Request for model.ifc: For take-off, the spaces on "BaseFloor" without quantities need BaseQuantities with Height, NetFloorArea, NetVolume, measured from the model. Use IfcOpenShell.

First a look at what the model holds.

```python
import ifcopenshell
import ifcopenshell.util.element
import ifcopenshell.util.unit

model = ifcopenshell.open("model.ifc")
print(model.schema)
for unit_type in ("LENGTHUNIT", "AREAUNIT", "VOLUMEUNIT"):
    print(unit_type, ifcopenshell.util.unit.calculate_unit_scale(model, unit_type))
storey = next(s for s in model.by_type("IfcBuildingStorey") if s.Name == "BaseFloor")
spaces = [e for e in ifcopenshell.util.element.get_decomposition(storey) if e.is_a("IfcSpace")]
for e in sorted(spaces, key=lambda e: e.id()):
    print(e.id(), e.is_a(), e.Name, list(ifcopenshell.util.element.get_psets(e, qtos_only=True)), sep=" | ")
```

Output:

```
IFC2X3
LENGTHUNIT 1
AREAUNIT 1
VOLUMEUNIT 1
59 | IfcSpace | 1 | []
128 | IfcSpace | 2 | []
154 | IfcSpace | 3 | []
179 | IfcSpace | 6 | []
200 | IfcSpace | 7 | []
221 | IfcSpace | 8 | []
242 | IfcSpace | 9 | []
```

```python
import ifcopenshell
import ifcopenshell.api.pset
import ifcopenshell.geom
import ifcopenshell.util.element
import ifcopenshell.util.shape
import ifcopenshell.util.unit

model = ifcopenshell.open("model.ifc")
unit_scale = ifcopenshell.util.unit.calculate_unit_scale(model)
area_scale = ifcopenshell.util.unit.calculate_unit_scale(model, "AREAUNIT")
volume_scale = ifcopenshell.util.unit.calculate_unit_scale(model, "VOLUMEUNIT")
settings = ifcopenshell.geom.settings()

storey = next(s for s in model.by_type("IfcBuildingStorey") if s.Name == "BaseFloor")
spaces = [e for e in ifcopenshell.util.element.get_decomposition(storey) if e.is_a("IfcSpace")]

for e in sorted(spaces, key=lambda e: e.id()):
    if ifcopenshell.util.element.get_psets(e, qtos_only=True, should_inherit=False):
        continue
    # Geometry comes back in metres, in the element's own axes.
    shape = ifcopenshell.geom.create_shape(settings, e)
    values = {
        "Height": ifcopenshell.util.shape.get_z(shape.geometry) / unit_scale,
        "NetFloorArea": ifcopenshell.util.shape.get_footprint_area(shape.geometry) / area_scale,
        "NetVolume": ifcopenshell.util.shape.get_volume(shape.geometry) / volume_scale,
    }
    qto = ifcopenshell.api.pset.add_qto(model, product=e, name="BaseQuantities")
    ifcopenshell.api.pset.edit_qto(model, qto=qto, properties=values)
    print(e.id(), {k: round(v, 3) for k, v in values.items()})

model.write("model-out.ifc")
```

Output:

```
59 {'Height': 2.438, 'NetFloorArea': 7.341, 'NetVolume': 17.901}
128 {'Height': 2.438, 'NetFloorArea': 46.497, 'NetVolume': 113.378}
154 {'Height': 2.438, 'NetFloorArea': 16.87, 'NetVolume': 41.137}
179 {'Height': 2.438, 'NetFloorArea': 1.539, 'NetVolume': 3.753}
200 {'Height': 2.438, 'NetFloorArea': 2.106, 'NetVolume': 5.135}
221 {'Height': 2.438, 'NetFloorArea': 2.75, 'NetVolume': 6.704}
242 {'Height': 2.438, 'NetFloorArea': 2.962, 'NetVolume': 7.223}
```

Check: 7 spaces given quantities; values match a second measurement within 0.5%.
